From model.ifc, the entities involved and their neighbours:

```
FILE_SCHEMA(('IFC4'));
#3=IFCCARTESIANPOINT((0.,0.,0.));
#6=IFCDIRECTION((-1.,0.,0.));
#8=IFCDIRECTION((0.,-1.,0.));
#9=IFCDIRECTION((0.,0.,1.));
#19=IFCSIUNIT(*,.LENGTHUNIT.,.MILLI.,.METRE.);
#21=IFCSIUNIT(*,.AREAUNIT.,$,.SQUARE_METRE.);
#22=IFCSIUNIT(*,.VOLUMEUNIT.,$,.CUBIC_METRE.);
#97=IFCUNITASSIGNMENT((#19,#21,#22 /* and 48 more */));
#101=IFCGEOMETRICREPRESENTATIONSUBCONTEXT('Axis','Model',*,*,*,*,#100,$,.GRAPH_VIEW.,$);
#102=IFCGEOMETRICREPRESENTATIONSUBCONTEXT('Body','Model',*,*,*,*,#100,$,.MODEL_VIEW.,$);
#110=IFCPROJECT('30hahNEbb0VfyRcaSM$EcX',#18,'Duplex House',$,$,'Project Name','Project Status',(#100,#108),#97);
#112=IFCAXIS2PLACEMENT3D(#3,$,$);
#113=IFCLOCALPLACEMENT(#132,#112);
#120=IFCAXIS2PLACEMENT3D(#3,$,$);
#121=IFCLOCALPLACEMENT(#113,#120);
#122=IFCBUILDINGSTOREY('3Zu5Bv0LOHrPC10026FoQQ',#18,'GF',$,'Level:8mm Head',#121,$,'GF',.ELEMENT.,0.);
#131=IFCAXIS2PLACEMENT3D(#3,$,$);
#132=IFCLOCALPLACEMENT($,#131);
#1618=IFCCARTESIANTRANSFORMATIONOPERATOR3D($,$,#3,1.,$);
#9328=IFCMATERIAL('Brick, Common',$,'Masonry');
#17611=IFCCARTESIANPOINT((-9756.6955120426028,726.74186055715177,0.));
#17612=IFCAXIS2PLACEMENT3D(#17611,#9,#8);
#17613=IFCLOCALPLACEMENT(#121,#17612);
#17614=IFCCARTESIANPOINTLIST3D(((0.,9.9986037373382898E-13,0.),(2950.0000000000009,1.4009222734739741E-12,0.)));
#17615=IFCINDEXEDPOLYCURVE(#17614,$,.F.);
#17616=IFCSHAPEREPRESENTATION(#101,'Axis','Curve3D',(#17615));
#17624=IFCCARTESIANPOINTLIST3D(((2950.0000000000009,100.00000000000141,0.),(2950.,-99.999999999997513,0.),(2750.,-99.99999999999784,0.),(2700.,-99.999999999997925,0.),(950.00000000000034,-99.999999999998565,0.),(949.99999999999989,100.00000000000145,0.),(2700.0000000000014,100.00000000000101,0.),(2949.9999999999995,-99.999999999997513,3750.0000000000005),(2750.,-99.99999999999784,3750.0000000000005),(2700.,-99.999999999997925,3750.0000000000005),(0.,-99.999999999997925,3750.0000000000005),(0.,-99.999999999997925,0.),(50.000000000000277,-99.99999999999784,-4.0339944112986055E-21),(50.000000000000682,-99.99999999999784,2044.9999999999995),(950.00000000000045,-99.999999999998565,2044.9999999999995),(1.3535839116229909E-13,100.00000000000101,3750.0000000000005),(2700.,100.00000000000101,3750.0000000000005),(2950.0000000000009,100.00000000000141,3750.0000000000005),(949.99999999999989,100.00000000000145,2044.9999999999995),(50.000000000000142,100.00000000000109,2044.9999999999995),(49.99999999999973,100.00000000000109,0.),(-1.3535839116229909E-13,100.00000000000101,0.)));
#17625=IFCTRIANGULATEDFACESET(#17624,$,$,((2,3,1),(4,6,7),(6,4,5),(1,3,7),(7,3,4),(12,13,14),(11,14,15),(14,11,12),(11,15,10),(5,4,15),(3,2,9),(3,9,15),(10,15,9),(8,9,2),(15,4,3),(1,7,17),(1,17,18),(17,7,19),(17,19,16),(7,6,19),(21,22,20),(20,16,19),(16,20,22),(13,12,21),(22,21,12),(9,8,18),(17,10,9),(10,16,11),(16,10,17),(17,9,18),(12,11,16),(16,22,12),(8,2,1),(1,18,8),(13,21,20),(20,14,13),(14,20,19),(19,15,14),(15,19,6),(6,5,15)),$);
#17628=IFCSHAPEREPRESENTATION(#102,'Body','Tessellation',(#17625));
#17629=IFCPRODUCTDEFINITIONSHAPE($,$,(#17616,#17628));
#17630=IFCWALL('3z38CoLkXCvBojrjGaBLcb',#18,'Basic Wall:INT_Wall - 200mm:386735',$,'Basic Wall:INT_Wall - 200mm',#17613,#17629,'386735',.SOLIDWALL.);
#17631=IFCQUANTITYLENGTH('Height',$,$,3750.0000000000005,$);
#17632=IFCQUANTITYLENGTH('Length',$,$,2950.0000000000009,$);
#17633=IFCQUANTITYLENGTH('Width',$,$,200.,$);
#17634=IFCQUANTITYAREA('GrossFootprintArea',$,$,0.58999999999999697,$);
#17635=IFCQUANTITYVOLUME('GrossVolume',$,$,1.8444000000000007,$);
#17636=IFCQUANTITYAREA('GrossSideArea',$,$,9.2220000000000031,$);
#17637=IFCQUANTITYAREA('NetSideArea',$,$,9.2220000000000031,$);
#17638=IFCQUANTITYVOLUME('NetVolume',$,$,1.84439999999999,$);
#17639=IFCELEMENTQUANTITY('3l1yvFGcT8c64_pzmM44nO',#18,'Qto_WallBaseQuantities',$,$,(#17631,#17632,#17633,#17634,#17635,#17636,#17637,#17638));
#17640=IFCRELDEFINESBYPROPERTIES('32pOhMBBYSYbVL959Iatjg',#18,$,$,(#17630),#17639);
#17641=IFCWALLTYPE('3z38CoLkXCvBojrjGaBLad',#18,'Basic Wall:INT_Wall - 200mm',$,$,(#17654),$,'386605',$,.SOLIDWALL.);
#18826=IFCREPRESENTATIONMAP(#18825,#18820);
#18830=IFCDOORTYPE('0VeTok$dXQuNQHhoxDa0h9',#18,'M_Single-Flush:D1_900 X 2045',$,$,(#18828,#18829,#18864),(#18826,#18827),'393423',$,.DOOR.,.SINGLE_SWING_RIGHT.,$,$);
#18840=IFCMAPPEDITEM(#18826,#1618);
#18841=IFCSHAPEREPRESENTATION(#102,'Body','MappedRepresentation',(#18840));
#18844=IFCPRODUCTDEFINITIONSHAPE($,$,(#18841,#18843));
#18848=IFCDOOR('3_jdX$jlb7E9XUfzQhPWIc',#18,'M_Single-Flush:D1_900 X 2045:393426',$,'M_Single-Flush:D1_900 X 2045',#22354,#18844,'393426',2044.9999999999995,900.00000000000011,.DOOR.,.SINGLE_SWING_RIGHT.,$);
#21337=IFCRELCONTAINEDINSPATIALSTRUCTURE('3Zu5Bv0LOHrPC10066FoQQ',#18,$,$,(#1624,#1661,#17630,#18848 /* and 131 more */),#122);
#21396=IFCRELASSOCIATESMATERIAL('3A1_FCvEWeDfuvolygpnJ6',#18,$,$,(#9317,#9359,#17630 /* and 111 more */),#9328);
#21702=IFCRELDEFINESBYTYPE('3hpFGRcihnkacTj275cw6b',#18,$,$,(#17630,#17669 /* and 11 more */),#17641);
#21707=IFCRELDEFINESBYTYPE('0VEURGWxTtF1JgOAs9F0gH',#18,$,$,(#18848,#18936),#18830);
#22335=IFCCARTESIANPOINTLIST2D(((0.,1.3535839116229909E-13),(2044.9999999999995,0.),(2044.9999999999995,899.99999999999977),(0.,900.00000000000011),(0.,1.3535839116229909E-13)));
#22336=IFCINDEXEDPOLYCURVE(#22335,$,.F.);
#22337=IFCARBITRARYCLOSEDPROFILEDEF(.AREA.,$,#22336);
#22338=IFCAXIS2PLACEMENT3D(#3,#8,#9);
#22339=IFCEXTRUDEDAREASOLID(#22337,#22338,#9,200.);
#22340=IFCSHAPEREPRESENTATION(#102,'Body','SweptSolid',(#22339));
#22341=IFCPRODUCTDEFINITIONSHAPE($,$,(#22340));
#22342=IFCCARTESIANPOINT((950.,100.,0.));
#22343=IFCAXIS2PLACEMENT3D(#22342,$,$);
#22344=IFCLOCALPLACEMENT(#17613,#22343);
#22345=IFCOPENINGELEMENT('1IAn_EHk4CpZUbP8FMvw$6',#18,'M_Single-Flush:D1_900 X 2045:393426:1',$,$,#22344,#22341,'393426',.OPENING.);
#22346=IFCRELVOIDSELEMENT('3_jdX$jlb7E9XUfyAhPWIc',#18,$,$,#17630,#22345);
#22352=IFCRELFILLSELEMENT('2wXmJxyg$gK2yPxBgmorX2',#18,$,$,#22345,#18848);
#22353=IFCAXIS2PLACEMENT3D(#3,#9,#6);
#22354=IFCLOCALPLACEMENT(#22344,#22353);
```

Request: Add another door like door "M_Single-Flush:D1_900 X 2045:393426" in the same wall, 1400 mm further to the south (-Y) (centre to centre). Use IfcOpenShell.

```python
import ifcopenshell
import ifcopenshell.api.feature
import ifcopenshell.api.geometry
import ifcopenshell.api.pset
import ifcopenshell.api.root
import ifcopenshell.geom
import ifcopenshell.util.element
import ifcopenshell.util.placement
import ifcopenshell.util.shape
import ifcopenshell.util.unit

model = ifcopenshell.open("model.ifc")
unit_scale = ifcopenshell.util.unit.calculate_unit_scale(model)
area_scale = ifcopenshell.util.unit.calculate_unit_scale(model, "AREAUNIT")
volume_scale = ifcopenshell.util.unit.calculate_unit_scale(model, "VOLUMEUNIT")
settings = ifcopenshell.geom.settings()


def volume(element):
    """Net volume in cubic metres, openings subtracted."""
    shape = ifcopenshell.geom.create_shape(settings, element)
    return ifcopenshell.util.shape.get_volume(shape.geometry)


def reuse_history(source, copy):
    """copy_class also copies each property set's owner history, people and application; keep the originals."""
    for rel in copy.IsDefinedBy:
        if rel.is_a("IfcRelDefinesByProperties") and (history := rel.RelatingPropertyDefinition.OwnerHistory):
            rel.RelatingPropertyDefinition.OwnerHistory = source.OwnerHistory
            ifcopenshell.util.element.remove_deep2(model, history)


door = model.by_guid("3_jdX$jlb7E9XUfzQhPWIc")
opening = door.FillsVoids[0].RelatingOpeningElement
wall = opening.VoidsElements[0].RelatingBuildingElement
before = volume(wall)
shift = ifcopenshell.util.placement.get_local_placement(wall.ObjectPlacement)[:3, 0] * 1.4 / unit_scale

# copy_class copies the void relationship, type, container and properties, but no geometry.
new_opening = ifcopenshell.api.root.copy_class(model, product=opening)
new_opening.Representation = ifcopenshell.util.element.copy_deep(
    model, opening.Representation, exclude=["IfcGeometricRepresentationContext", "IfcRepresentationMap"]
)
new_opening.Name = "M_Single-Flush:D1_900 X 2045"
new_opening.Tag = None
reuse_history(opening, new_opening)
new_door = ifcopenshell.api.root.copy_class(model, product=door)
new_door.Representation = ifcopenshell.util.element.copy_deep(
    model, door.Representation, exclude=["IfcGeometricRepresentationContext", "IfcRepresentationMap"]
)
new_door.Name = "M_Single-Flush:D1_900 X 2045"
new_door.Tag = None
reuse_history(door, new_door)
ifcopenshell.api.feature.add_filling(model, opening=new_opening, element=new_door)

for old, new in ((opening, new_opening), (door, new_door)):
    matrix = ifcopenshell.util.placement.get_local_placement(old.ObjectPlacement)
    matrix[:3, 3] += shift
    ifcopenshell.api.geometry.edit_object_placement(model, product=new, matrix=matrix, is_si=False)

after = volume(wall)
thickness = 0.2  # wall thickness in metres

# Update the wall's stored quantities.
qto = model.by_id(ifcopenshell.util.element.get_pset(wall, "Qto_WallBaseQuantities", should_inherit=False)["id"])
ifcopenshell.api.pset.edit_qto(model, qto=qto, properties={
    "NetSideArea": after / thickness / area_scale,
    "NetVolume": after / volume_scale,
})

print(f"wall volume {before:.3f} -> {after:.3f} m3")

model.write("model-out.ifc")
```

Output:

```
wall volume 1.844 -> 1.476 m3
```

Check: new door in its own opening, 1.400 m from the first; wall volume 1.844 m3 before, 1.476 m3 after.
